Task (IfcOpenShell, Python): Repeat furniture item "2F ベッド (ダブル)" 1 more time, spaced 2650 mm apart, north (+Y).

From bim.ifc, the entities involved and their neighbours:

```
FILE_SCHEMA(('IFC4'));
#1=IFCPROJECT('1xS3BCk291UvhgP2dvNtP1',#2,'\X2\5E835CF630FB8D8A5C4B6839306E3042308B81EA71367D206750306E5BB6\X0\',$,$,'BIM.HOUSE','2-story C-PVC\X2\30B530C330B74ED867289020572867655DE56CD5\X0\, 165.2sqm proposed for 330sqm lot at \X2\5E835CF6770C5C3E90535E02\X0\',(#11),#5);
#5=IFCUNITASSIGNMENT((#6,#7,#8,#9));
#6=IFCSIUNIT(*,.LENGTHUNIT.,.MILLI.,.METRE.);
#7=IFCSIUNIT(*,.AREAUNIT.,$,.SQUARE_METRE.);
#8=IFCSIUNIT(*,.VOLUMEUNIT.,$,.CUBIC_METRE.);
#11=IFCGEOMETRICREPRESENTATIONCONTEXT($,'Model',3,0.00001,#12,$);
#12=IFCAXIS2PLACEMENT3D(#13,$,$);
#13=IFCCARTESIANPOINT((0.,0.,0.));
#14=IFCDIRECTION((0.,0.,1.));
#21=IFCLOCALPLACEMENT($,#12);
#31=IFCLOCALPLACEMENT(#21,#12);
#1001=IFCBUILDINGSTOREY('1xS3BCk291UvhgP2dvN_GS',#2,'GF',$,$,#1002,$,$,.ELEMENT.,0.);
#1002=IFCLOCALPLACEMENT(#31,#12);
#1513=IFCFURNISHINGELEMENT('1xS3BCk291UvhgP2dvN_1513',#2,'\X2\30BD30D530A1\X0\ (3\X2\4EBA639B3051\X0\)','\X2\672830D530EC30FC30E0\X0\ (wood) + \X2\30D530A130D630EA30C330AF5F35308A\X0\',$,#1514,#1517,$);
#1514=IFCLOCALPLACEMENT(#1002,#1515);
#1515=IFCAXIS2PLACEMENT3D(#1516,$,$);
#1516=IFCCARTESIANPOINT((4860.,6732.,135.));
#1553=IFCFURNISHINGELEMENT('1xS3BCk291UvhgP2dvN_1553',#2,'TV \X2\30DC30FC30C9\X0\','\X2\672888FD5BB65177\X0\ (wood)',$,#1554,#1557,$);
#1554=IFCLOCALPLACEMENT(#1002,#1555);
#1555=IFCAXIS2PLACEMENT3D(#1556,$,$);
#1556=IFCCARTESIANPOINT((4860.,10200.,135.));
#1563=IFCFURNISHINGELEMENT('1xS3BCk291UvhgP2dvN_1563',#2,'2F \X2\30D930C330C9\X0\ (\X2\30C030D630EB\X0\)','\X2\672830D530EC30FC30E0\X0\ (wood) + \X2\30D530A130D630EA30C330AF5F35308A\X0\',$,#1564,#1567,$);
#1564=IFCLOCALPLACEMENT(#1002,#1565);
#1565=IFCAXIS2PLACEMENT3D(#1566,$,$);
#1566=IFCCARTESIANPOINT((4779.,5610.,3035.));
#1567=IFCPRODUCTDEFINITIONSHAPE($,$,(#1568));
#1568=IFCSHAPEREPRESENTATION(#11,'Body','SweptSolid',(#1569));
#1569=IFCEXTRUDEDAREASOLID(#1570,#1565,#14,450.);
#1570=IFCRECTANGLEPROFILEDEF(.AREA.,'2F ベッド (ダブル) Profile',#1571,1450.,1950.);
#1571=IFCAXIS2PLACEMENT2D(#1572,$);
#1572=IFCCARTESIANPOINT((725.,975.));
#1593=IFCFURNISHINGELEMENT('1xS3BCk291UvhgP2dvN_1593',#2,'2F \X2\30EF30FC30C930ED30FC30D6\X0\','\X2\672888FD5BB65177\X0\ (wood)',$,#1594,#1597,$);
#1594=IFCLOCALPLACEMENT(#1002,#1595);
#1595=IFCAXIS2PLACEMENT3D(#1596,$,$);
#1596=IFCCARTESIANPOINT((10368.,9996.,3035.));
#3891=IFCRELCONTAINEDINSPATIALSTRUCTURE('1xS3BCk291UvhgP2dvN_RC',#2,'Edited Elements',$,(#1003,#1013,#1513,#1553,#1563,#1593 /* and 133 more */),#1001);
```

```python
import numpy as np
import ifcopenshell
import ifcopenshell.api.geometry
import ifcopenshell.api.root
import ifcopenshell.util.element
import ifcopenshell.util.placement
import ifcopenshell.util.unit

model = ifcopenshell.open("bim.ifc")
unit_scale = ifcopenshell.util.unit.calculate_unit_scale(model)


def reuse_history(source, copy):
    """copy_class also copies each property set's owner history, people and application; keep the originals."""
    for rel in copy.IsDefinedBy:
        if rel.is_a("IfcRelDefinesByProperties") and (history := rel.RelatingPropertyDefinition.OwnerHistory):
            rel.RelatingPropertyDefinition.OwnerHistory = source.OwnerHistory
            ifcopenshell.util.element.remove_deep2(model, history)


source = model.by_id(1563)
base = ifcopenshell.util.placement.get_local_placement(source.ObjectPlacement)
step = np.array([0.0, 1.0, 0.0]) * 2.65 / unit_scale

for i in range(1, 2):
    copy = ifcopenshell.api.root.copy_class(model, product=source)
    copy.Representation = ifcopenshell.util.element.copy_deep(
        model, source.Representation, exclude=["IfcGeometricRepresentationContext", "IfcRepresentationMap"]
    )
    reuse_history(source, copy)
    matrix = base.copy()
    matrix[:3, 3] += i * step
    print("added at", matrix[:3, 3].round(3) + 0.0)
    ifcopenshell.api.geometry.edit_object_placement(model, product=copy, matrix=matrix, is_si=False)

model.write("bim_edited.ifc")
```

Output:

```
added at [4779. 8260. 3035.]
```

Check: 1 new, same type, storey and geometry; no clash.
